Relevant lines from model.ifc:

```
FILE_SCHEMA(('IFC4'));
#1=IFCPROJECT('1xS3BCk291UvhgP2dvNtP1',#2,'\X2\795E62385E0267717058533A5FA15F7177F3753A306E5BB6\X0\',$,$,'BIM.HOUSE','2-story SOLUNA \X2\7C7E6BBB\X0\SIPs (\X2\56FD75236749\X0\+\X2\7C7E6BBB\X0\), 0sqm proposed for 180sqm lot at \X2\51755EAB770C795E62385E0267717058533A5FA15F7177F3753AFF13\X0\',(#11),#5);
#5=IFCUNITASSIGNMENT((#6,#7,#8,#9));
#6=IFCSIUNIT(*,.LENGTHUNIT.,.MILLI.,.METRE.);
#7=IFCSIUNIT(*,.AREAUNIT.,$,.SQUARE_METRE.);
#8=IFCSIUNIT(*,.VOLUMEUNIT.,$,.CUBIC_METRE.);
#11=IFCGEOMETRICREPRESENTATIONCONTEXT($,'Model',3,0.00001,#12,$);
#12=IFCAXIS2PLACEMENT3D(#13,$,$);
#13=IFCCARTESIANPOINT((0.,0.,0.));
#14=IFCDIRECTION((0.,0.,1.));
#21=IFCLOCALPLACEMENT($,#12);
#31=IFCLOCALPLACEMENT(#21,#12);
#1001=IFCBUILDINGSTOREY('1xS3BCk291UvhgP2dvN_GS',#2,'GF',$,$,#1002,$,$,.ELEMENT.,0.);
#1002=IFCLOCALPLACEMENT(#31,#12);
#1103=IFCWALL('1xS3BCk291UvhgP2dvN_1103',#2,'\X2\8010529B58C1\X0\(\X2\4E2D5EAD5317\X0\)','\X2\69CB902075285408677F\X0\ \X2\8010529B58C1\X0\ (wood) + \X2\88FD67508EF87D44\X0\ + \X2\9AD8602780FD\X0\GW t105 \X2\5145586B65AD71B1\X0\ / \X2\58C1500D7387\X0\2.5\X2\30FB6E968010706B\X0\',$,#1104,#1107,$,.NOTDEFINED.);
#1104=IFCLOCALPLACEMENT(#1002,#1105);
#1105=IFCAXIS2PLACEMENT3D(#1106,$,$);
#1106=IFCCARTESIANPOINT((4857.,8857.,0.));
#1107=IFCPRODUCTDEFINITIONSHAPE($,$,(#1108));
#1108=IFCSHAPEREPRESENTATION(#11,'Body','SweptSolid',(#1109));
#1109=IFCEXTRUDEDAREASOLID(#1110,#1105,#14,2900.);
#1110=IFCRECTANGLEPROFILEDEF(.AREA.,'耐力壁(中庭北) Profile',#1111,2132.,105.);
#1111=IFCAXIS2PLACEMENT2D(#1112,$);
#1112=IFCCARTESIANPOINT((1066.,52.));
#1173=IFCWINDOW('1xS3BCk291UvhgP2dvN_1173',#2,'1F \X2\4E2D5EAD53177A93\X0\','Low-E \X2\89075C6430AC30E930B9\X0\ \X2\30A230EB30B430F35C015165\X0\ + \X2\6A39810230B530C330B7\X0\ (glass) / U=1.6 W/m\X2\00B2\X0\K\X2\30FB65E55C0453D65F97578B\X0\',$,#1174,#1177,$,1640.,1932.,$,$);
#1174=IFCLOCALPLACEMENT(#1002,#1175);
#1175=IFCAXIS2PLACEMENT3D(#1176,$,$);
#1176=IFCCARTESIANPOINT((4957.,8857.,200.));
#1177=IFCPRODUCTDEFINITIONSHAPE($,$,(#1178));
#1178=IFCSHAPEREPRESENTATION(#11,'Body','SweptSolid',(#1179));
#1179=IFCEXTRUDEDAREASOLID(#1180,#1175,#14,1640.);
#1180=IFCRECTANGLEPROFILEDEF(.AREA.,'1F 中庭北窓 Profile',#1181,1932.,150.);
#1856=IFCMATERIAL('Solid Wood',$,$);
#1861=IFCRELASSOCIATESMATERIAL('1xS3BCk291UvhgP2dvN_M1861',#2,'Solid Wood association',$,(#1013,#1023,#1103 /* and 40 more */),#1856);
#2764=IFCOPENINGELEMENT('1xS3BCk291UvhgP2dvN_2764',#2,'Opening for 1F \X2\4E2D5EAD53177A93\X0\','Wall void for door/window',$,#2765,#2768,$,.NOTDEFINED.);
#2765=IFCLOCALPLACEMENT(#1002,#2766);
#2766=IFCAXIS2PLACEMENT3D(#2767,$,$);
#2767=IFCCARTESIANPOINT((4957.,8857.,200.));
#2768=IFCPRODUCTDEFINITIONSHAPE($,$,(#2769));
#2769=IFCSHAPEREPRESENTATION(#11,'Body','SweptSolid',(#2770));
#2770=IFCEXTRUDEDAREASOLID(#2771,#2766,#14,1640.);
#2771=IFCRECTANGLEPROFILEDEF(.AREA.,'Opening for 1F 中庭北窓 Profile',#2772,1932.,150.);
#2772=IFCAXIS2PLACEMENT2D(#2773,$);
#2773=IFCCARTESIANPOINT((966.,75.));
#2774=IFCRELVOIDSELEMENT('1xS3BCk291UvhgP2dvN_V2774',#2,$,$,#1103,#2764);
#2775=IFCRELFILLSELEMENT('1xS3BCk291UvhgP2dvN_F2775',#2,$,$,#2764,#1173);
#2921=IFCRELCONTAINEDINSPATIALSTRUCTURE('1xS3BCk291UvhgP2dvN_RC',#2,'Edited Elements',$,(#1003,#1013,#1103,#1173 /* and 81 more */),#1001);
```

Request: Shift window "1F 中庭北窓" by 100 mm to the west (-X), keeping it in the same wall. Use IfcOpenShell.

```python
import ifcopenshell
import ifcopenshell.api.geometry
import ifcopenshell.util.placement

model = ifcopenshell.open("model.ifc")

window = model.by_guid("1xS3BCk291UvhgP2dvN_1173")
opening = window.FillsVoids[0].RelatingOpeningElement
wall = opening.VoidsElements[0].RelatingBuildingElement

wall_matrix = ifcopenshell.util.placement.get_local_placement(wall.ObjectPlacement)
shift = wall_matrix[:3, 0] * -100.0
before = ifcopenshell.util.placement.get_local_placement(window.ObjectPlacement)[:3, 3].copy()

# The window is not placed relative to its opening, so move both.
for product in (opening, window):
    matrix = ifcopenshell.util.placement.get_local_placement(product.ObjectPlacement)
    matrix[:3, 3] += shift
    ifcopenshell.api.geometry.edit_object_placement(model, product=product, matrix=matrix, is_si=False)

after = ifcopenshell.util.placement.get_local_placement(window.ObjectPlacement)[:3, 3]
print("window moved by", (after - before).round(3) + 0.0)

model.write("model-out.ifc")
```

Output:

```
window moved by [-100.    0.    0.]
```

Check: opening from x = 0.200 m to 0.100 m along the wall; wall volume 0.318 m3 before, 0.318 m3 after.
